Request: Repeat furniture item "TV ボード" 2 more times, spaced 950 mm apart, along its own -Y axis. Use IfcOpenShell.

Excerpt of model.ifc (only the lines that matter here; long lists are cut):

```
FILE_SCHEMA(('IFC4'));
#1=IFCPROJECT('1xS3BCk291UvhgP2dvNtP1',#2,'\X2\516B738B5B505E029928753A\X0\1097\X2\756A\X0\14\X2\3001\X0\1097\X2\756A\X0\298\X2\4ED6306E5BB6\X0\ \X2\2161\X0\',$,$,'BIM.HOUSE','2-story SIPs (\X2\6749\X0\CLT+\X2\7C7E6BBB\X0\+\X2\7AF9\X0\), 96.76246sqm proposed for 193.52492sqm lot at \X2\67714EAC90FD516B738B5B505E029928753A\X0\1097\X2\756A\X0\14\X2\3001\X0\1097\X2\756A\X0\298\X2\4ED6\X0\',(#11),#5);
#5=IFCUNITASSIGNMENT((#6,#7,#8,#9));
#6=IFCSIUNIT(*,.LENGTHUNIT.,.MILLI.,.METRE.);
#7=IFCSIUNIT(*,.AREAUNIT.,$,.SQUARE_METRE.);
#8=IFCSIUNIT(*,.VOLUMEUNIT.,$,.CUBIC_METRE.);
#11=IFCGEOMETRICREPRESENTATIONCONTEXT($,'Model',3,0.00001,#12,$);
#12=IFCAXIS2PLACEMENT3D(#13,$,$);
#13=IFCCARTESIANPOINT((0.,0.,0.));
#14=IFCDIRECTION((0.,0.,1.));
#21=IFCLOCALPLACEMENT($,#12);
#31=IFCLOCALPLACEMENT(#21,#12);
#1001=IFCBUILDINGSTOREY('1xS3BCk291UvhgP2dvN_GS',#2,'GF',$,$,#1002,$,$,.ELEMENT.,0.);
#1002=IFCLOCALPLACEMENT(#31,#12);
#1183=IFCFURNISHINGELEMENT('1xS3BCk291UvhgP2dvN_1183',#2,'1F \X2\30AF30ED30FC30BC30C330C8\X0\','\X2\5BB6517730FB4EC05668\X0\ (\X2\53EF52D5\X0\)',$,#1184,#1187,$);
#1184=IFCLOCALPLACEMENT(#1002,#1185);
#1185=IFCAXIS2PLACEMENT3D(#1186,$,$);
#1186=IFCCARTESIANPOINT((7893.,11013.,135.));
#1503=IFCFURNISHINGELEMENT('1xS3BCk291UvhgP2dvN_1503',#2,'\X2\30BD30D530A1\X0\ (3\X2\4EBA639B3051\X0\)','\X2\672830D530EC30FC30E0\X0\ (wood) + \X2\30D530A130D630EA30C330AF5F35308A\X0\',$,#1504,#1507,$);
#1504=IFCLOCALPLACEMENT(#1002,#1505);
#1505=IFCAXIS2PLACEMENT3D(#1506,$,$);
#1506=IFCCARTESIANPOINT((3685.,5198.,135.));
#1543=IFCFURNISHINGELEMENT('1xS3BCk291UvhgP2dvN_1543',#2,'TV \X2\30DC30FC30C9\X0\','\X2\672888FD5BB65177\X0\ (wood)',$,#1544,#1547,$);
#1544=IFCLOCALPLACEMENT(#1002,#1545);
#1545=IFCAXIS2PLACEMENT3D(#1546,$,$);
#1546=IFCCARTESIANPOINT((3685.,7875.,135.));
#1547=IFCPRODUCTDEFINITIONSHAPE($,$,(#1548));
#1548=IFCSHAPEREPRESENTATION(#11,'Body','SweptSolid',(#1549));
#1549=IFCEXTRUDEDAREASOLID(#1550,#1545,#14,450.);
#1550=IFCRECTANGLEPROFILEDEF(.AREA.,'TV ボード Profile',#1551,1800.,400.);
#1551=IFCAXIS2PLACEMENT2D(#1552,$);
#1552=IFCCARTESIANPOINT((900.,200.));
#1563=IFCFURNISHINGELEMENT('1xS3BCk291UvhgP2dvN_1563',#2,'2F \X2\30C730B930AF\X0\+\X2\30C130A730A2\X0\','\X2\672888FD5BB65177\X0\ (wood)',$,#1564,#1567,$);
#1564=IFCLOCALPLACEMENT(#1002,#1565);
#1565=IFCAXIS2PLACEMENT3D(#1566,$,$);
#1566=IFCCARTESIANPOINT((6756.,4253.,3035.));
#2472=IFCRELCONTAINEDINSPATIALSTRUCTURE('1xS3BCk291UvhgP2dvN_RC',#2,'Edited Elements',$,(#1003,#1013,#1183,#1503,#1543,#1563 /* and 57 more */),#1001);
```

```python
import ifcopenshell
import ifcopenshell.api.geometry
import ifcopenshell.api.root
import ifcopenshell.util.element
import ifcopenshell.util.placement

model = ifcopenshell.open("model.ifc")


def reuse_history(source, copy):
    """copy_class also copies each property set's owner history, people and application; keep the originals."""
    for rel in copy.IsDefinedBy:
        if rel.is_a("IfcRelDefinesByProperties") and (history := rel.RelatingPropertyDefinition.OwnerHistory):
            rel.RelatingPropertyDefinition.OwnerHistory = source.OwnerHistory
            ifcopenshell.util.element.remove_deep2(model, history)


source = model.by_guid("1xS3BCk291UvhgP2dvN_1543")
base = ifcopenshell.util.placement.get_local_placement(source.ObjectPlacement)
step = -base[:3, 1] * 950.0

for i in range(1, 3):
    copy = ifcopenshell.api.root.copy_class(model, product=source)
    copy.Representation = ifcopenshell.util.element.copy_deep(
        model, source.Representation, exclude=["IfcGeometricRepresentationContext", "IfcRepresentationMap"]
    )
    reuse_history(source, copy)
    matrix = base.copy()
    matrix[:3, 3] += i * step
    print("added at", matrix[:3, 3].round(3) + 0.0)
    ifcopenshell.api.geometry.edit_object_placement(model, product=copy, matrix=matrix, is_si=False)

model.write("model_v2.ifc")
```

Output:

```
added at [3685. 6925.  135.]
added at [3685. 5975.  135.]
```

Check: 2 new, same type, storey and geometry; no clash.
